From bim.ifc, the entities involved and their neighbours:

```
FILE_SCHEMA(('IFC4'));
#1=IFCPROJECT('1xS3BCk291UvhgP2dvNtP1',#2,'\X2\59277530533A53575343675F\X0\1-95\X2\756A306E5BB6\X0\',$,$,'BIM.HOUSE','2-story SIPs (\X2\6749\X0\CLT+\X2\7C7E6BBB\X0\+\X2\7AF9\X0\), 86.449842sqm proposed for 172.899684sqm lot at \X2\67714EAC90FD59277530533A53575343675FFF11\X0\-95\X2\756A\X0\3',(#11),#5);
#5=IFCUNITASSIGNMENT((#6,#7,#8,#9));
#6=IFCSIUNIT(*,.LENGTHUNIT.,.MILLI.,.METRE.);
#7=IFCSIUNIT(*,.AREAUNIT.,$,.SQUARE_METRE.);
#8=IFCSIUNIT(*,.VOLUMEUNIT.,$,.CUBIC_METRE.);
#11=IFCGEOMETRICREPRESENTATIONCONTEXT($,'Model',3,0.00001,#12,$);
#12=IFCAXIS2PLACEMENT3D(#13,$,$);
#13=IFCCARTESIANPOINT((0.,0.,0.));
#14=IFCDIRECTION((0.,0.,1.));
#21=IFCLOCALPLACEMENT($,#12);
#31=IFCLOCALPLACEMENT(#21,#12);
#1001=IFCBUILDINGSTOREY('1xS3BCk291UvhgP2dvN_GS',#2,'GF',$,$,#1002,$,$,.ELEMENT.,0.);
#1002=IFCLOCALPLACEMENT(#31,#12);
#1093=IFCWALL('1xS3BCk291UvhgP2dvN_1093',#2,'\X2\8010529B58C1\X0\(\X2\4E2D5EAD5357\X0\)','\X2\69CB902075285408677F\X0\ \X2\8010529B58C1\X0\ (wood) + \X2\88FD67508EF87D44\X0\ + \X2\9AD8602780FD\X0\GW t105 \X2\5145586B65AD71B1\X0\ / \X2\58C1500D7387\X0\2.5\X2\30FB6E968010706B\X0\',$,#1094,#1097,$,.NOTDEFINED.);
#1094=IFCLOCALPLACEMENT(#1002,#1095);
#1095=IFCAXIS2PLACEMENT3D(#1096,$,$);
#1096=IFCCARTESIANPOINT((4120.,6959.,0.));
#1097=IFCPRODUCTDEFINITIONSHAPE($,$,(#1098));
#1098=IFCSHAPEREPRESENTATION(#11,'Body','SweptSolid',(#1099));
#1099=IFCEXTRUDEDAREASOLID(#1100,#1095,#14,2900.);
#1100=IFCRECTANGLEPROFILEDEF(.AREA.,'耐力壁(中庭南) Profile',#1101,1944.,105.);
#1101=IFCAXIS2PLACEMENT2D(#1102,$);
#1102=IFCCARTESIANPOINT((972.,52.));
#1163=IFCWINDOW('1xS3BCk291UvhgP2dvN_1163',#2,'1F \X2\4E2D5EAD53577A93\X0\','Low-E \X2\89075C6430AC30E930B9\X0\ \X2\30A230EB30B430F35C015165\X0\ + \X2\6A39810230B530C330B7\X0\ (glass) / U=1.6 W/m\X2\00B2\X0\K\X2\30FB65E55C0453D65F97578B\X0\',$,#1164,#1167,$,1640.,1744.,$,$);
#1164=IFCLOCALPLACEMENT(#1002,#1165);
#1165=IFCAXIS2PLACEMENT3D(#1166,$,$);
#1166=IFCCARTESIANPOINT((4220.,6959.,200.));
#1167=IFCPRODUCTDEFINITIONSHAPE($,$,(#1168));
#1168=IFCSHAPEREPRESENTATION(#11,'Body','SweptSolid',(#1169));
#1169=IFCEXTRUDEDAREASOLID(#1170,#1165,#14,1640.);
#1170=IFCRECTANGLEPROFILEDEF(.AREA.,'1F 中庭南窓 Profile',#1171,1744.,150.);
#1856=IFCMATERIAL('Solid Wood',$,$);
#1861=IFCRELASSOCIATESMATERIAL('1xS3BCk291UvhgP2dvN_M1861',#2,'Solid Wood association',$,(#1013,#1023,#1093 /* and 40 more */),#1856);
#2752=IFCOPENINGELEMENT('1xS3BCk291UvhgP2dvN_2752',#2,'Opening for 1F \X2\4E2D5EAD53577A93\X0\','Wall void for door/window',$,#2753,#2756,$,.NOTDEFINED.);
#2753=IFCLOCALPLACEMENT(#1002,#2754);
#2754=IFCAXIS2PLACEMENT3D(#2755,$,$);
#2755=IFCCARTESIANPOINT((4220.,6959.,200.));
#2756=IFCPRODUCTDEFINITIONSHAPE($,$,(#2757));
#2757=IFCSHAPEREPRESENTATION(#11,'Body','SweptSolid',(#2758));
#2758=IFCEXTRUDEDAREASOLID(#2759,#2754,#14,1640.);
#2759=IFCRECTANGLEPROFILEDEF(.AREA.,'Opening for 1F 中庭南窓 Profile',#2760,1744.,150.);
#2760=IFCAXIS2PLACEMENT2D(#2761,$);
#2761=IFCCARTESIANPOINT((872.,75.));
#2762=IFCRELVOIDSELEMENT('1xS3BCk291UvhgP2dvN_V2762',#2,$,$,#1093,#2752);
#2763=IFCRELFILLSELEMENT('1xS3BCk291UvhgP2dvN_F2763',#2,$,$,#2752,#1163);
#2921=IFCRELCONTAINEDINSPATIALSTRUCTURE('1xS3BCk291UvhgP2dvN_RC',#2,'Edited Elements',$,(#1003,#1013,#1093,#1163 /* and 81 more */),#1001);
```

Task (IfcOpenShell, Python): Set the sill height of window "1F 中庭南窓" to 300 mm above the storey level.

```python
import numpy as np
import ifcopenshell
import ifcopenshell.api.geometry
import ifcopenshell.geom
import ifcopenshell.util.element
import ifcopenshell.util.placement
import ifcopenshell.util.shape
import ifcopenshell.util.unit

model = ifcopenshell.open("bim.ifc")
unit_scale = ifcopenshell.util.unit.calculate_unit_scale(model)

window = model.by_id(1163)
opening = window.FillsVoids[0].RelatingOpeningElement
storey = ifcopenshell.util.element.get_container(window, ifc_class="IfcBuildingStorey")
level = ifcopenshell.util.placement.get_local_placement(storey.ObjectPlacement)[2, 3]

# The opening's origin need not be at the sill, so measure its lowest point.
shape = ifcopenshell.geom.create_shape(ifcopenshell.geom.settings(), opening)
bottom = ifcopenshell.util.shape.get_shape_bottom_elevation(shape, shape.geometry) / unit_scale
dz = level + 0.3 / unit_scale - bottom

shift = np.array([0.0, 0.0, dz])
# The window is not placed relative to its opening, so move both.
for product in (opening, window):
    matrix = ifcopenshell.util.placement.get_local_placement(product.ObjectPlacement)
    matrix[:3, 3] += shift
    ifcopenshell.api.geometry.edit_object_placement(model, product=product, matrix=matrix, is_si=False)

print(f"moved by {dz * unit_scale:+.3f} m")

model.write("bim_updated.ifc")
```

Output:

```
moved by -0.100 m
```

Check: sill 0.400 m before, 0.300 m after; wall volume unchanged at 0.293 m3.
